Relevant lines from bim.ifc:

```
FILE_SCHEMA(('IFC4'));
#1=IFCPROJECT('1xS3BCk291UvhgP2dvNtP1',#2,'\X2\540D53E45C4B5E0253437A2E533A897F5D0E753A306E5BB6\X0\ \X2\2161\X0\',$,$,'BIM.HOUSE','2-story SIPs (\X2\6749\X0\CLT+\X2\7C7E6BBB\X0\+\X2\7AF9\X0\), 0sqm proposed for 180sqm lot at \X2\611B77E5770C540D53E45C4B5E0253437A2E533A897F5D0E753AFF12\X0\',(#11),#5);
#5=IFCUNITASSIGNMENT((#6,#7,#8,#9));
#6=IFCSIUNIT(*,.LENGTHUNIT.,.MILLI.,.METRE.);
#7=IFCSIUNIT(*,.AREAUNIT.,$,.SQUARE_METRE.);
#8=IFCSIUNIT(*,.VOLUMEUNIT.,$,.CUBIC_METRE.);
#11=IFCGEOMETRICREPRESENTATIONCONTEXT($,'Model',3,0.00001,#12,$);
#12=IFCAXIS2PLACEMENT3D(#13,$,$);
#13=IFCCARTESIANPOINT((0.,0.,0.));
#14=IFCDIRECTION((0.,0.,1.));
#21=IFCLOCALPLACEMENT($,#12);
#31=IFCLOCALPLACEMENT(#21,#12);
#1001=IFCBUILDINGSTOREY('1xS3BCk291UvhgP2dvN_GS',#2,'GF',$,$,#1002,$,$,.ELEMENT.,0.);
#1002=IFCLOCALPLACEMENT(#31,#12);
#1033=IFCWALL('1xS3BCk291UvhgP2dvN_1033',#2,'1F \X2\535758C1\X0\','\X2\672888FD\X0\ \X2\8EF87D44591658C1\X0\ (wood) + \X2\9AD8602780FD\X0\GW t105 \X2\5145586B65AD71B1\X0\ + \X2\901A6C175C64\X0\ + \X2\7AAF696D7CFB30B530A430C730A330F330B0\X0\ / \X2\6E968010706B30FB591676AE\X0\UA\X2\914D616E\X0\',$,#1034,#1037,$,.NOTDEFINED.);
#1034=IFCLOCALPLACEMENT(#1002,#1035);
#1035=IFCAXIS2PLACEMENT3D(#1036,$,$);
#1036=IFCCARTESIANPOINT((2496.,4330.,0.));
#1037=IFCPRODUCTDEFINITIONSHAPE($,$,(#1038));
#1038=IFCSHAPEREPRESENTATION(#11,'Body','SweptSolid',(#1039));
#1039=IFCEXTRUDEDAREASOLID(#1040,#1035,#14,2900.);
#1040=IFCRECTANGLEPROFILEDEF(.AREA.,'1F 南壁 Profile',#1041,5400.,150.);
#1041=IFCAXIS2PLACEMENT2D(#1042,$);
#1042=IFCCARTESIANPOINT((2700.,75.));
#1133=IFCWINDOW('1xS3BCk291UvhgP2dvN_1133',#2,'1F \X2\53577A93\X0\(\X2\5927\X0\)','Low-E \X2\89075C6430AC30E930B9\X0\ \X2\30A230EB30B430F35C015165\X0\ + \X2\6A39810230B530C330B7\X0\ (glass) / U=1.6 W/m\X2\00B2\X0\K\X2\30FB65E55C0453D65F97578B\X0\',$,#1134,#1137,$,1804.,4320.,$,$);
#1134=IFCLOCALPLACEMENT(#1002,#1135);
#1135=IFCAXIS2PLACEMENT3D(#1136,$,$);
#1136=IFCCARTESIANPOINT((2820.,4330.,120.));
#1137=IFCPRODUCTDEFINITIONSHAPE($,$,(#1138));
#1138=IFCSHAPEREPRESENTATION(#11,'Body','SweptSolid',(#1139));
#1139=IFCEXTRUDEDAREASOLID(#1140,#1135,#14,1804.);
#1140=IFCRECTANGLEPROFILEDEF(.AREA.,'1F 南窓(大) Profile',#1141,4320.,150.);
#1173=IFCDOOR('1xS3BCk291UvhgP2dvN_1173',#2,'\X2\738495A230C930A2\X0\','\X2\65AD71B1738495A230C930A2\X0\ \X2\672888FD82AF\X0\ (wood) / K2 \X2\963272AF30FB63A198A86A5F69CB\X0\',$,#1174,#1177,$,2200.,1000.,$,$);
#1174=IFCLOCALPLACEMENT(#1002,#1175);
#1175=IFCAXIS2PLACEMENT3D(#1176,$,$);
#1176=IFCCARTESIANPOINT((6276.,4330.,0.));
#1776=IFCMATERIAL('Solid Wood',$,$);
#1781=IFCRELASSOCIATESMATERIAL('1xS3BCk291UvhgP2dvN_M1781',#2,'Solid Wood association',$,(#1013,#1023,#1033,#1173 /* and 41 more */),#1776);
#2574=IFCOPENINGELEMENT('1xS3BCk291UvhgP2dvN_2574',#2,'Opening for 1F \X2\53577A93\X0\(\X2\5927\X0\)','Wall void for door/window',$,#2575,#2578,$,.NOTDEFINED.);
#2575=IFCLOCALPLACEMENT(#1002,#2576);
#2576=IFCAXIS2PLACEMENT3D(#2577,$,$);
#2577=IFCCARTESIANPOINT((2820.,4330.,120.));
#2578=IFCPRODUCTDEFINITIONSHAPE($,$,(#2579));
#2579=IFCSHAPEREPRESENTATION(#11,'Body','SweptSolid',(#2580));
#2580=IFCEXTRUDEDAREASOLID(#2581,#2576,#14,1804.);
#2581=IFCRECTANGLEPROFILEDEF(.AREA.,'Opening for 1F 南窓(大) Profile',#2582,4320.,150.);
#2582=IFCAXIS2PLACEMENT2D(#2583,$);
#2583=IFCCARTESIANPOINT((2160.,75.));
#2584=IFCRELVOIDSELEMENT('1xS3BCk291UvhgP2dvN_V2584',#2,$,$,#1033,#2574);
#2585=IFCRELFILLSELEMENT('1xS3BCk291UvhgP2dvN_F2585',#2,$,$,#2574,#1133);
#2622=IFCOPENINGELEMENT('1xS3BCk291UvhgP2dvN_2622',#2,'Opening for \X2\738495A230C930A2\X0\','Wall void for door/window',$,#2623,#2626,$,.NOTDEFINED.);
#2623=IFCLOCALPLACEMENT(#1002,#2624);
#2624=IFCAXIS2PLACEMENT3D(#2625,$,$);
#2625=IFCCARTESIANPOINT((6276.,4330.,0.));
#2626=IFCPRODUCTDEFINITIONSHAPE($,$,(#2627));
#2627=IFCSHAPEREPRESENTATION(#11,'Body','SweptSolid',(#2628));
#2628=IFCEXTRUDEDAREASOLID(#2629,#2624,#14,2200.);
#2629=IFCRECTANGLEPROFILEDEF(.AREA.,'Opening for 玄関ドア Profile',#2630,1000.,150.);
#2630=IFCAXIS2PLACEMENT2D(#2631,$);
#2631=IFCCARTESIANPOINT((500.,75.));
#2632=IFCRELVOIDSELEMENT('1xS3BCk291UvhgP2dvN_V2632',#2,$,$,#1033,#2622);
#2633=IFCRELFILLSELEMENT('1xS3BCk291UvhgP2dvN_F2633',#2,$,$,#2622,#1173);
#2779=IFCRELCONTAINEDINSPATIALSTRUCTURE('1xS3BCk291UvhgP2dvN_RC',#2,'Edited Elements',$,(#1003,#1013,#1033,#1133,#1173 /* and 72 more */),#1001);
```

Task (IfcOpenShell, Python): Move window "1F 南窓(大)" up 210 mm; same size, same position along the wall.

```python
import numpy as np
import ifcopenshell
import ifcopenshell.api.geometry
import ifcopenshell.util.placement
import ifcopenshell.util.unit

model = ifcopenshell.open("bim.ifc")
unit_scale = ifcopenshell.util.unit.calculate_unit_scale(model)

window = model.by_guid("1xS3BCk291UvhgP2dvN_1133")
opening = window.FillsVoids[0].RelatingOpeningElement
dz = 0.21 / unit_scale

shift = np.array([0.0, 0.0, dz])
# The window is not placed relative to its opening, so move both.
for product in (opening, window):
    matrix = ifcopenshell.util.placement.get_local_placement(product.ObjectPlacement)
    matrix[:3, 3] += shift
    ifcopenshell.api.geometry.edit_object_placement(model, product=product, matrix=matrix, is_si=False)

print(f"moved by {dz * unit_scale:+.3f} m")

model.write("bim_rev.ifc")
```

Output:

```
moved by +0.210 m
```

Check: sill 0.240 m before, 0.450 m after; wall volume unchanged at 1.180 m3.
